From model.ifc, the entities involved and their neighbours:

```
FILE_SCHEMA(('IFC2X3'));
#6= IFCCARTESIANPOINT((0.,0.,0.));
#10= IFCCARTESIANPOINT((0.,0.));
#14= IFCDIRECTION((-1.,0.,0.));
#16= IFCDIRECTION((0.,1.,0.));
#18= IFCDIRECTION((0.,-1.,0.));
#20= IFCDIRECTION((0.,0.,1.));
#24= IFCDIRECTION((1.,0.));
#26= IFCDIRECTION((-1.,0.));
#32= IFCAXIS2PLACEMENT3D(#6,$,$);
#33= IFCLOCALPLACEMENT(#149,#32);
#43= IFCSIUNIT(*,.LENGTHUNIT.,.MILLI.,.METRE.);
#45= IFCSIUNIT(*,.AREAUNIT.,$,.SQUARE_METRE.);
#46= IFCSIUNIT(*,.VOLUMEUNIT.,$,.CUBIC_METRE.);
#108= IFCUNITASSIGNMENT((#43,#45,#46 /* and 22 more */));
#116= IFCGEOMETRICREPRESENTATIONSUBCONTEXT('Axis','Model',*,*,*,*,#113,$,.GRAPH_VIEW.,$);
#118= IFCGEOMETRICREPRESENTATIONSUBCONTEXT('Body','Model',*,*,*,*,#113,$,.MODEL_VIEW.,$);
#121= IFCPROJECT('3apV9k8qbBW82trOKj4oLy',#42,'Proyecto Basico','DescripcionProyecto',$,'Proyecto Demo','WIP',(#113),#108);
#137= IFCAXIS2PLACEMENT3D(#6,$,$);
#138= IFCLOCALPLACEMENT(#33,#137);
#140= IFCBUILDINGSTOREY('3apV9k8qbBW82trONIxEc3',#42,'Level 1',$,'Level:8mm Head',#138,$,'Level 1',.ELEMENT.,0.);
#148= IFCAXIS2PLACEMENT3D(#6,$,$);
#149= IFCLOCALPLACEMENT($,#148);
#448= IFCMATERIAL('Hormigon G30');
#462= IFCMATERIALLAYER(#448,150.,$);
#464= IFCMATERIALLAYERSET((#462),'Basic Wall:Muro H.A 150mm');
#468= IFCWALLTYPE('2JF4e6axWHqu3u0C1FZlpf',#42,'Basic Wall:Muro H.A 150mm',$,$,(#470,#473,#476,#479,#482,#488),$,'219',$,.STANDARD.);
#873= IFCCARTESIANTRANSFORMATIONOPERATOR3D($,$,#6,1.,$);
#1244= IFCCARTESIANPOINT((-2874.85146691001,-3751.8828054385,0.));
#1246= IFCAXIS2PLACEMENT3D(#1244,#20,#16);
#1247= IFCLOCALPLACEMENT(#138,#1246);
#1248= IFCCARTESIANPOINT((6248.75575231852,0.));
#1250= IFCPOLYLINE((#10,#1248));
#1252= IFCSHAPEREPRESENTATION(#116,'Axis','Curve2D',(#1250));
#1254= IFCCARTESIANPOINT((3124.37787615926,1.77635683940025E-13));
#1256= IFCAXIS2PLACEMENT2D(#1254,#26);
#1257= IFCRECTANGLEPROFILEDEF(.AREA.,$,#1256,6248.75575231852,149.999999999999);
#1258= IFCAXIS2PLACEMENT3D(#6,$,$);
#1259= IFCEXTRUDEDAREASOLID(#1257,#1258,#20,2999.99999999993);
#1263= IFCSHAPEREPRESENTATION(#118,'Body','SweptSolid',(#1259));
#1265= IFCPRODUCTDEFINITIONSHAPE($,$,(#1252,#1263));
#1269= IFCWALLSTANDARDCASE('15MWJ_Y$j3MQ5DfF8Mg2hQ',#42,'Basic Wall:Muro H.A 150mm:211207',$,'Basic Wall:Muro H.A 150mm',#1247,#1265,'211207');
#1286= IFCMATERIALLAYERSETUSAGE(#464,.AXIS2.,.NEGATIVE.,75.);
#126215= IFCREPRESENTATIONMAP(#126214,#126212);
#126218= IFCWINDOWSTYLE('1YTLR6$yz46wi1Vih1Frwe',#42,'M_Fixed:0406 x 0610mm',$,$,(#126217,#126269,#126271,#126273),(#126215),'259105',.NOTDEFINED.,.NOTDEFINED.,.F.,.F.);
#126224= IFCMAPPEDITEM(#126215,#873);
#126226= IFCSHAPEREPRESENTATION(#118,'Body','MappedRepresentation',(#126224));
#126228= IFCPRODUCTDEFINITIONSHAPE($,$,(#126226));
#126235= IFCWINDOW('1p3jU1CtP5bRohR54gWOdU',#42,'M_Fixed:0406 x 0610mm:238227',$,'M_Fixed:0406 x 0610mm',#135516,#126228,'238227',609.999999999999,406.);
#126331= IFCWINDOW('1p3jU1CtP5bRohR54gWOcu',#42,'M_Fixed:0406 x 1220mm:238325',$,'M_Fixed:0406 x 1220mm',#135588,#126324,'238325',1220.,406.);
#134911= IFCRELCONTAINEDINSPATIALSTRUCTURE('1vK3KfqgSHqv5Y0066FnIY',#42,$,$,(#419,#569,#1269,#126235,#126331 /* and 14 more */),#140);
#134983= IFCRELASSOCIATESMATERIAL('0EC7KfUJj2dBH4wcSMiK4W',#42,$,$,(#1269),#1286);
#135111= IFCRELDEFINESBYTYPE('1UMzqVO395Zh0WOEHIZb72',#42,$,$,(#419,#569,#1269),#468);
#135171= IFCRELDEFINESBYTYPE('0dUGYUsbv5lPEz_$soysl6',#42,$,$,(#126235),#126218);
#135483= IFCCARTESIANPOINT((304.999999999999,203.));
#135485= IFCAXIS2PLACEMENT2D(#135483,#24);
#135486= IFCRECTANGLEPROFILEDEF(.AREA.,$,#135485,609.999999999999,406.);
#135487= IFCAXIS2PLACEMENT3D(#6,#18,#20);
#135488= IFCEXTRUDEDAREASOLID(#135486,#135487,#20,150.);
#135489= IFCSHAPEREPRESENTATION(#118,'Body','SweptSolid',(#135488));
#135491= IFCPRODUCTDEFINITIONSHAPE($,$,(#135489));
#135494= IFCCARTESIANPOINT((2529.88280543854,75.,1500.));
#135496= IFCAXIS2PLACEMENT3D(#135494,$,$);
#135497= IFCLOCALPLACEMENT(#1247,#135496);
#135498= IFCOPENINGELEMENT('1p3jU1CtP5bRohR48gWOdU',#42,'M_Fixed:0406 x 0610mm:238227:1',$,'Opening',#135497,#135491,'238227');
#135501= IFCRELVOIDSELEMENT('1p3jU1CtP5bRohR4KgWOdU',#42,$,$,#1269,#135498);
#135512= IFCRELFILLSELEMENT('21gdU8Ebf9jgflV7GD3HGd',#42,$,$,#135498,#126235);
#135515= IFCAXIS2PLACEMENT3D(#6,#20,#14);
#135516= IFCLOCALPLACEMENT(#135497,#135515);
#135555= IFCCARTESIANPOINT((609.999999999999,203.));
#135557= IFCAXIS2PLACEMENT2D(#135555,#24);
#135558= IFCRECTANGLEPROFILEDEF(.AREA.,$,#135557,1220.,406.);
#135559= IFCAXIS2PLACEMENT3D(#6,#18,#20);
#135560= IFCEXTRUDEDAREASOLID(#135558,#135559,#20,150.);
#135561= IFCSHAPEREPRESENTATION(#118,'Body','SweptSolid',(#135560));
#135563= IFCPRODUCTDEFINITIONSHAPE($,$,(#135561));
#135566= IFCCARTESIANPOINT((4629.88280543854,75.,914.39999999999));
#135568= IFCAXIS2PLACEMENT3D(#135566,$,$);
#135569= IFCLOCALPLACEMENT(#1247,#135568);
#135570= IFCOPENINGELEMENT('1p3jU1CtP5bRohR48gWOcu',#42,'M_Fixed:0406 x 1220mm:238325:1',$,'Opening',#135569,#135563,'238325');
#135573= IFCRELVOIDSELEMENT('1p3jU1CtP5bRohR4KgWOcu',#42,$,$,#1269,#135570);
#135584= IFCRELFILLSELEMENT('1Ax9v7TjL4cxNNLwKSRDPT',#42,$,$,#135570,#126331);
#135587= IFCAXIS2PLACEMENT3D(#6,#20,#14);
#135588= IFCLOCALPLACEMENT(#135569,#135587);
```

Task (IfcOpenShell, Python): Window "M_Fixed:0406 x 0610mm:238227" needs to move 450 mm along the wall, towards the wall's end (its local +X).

```python
import ifcopenshell
import ifcopenshell.api.geometry
import ifcopenshell.util.placement

model = ifcopenshell.open("model.ifc")

window = model.by_guid("1p3jU1CtP5bRohR54gWOdU")
opening = window.FillsVoids[0].RelatingOpeningElement
wall = opening.VoidsElements[0].RelatingBuildingElement

wall_matrix = ifcopenshell.util.placement.get_local_placement(wall.ObjectPlacement)
shift = wall_matrix[:3, 0] * 450.0
before = ifcopenshell.util.placement.get_local_placement(window.ObjectPlacement)[:3, 3].copy()

# The window is placed relative to its opening, so it follows when the opening moves.
matrix = ifcopenshell.util.placement.get_local_placement(opening.ObjectPlacement)
matrix[:3, 3] += shift
ifcopenshell.api.geometry.edit_object_placement(
    model, product=opening, matrix=matrix, is_si=False, should_transform_children=True
)

after = ifcopenshell.util.placement.get_local_placement(window.ObjectPlacement)[:3, 3]
print("window moved by", (after - before).round(3) + 0.0)

model.write("model_edited.ifc")
```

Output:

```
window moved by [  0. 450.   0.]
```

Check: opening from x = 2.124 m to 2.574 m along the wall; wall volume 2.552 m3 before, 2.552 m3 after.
